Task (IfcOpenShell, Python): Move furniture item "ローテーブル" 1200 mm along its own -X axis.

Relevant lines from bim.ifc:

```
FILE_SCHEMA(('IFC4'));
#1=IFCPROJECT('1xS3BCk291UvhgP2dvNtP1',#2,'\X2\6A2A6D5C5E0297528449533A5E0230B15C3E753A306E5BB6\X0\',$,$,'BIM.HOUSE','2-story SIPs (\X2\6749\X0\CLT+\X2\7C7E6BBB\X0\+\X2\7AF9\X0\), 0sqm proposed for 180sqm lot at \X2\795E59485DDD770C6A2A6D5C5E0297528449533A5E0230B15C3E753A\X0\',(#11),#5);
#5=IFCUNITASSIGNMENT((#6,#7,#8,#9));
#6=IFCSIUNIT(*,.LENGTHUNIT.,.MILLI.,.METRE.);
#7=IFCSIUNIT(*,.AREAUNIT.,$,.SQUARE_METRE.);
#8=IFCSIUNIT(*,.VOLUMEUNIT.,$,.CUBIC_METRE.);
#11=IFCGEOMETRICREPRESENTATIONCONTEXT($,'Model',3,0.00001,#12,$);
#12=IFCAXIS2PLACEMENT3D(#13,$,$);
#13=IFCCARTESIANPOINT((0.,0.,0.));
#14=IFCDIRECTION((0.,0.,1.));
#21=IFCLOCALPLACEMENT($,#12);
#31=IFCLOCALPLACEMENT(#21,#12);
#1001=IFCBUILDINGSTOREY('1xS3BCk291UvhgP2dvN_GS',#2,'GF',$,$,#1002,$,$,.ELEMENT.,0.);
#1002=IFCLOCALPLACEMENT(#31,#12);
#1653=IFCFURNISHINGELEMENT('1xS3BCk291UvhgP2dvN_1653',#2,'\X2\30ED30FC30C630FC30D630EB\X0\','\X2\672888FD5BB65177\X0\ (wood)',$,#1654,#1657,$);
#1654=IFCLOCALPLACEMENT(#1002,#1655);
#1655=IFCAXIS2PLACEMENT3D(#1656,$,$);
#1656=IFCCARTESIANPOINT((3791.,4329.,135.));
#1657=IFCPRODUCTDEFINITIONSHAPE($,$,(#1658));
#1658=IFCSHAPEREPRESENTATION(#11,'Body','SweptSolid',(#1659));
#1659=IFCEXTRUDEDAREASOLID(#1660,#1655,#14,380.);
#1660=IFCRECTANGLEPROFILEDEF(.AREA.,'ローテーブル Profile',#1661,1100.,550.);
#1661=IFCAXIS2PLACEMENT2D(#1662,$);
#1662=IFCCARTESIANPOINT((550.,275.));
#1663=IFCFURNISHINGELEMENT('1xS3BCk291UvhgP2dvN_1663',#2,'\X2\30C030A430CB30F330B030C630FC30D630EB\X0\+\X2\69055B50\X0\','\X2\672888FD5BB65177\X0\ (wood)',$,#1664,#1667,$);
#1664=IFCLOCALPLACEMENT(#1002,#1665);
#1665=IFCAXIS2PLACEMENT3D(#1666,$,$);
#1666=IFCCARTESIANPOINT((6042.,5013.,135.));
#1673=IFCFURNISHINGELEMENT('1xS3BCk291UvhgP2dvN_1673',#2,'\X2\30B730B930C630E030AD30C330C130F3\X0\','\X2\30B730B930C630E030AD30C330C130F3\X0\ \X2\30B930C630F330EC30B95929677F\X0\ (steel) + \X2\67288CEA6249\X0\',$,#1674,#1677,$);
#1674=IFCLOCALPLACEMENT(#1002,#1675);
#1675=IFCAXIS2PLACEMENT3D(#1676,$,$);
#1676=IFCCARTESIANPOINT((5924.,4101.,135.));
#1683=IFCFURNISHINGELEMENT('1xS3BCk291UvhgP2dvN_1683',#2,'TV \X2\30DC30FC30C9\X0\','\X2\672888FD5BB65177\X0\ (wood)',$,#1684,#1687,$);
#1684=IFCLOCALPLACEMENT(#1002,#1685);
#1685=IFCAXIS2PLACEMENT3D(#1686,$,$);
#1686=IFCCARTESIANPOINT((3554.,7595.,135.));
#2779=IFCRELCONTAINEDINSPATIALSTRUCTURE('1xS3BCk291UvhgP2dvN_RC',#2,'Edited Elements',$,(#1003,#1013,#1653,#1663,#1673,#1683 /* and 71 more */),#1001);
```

```python
import ifcopenshell
import ifcopenshell.api.geometry
import ifcopenshell.util.placement
import ifcopenshell.util.unit

model = ifcopenshell.open("bim.ifc")
unit_scale = ifcopenshell.util.unit.calculate_unit_scale(model)

item = model.by_guid("1xS3BCk291UvhgP2dvN_1653")
matrix = ifcopenshell.util.placement.get_local_placement(item.ObjectPlacement)
matrix[:3, 3] -= matrix[:3, 0] * 1.2 / unit_scale
ifcopenshell.api.geometry.edit_object_placement(model, product=item, matrix=matrix, is_si=False)

print(ifcopenshell.util.placement.get_local_placement(item.ObjectPlacement).round(3) + 0.0)

model.write("bim-out.ifc")
```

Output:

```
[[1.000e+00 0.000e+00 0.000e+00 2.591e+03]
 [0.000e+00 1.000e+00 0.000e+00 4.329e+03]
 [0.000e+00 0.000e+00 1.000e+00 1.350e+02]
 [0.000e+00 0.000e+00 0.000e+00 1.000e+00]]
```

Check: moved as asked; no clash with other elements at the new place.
